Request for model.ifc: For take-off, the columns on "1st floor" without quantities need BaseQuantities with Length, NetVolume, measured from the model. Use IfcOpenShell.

First a look at what the model holds.

```python
import ifcopenshell
import ifcopenshell.util.element
import ifcopenshell.util.unit

model = ifcopenshell.open("model.ifc")
print(model.schema)
for unit_type in ("LENGTHUNIT", "AREAUNIT", "VOLUMEUNIT"):
    print(unit_type, ifcopenshell.util.unit.calculate_unit_scale(model, unit_type))
storey = next(s for s in model.by_type("IfcBuildingStorey") if s.Name == "1st floor")
columns = [e for e in ifcopenshell.util.element.get_decomposition(storey) if e.is_a("IfcColumn")]
for e in sorted(columns, key=lambda e: e.id()):
    print(e.id(), e.is_a(), e.Name, list(ifcopenshell.util.element.get_psets(e, qtos_only=True)), sep=" | ")
```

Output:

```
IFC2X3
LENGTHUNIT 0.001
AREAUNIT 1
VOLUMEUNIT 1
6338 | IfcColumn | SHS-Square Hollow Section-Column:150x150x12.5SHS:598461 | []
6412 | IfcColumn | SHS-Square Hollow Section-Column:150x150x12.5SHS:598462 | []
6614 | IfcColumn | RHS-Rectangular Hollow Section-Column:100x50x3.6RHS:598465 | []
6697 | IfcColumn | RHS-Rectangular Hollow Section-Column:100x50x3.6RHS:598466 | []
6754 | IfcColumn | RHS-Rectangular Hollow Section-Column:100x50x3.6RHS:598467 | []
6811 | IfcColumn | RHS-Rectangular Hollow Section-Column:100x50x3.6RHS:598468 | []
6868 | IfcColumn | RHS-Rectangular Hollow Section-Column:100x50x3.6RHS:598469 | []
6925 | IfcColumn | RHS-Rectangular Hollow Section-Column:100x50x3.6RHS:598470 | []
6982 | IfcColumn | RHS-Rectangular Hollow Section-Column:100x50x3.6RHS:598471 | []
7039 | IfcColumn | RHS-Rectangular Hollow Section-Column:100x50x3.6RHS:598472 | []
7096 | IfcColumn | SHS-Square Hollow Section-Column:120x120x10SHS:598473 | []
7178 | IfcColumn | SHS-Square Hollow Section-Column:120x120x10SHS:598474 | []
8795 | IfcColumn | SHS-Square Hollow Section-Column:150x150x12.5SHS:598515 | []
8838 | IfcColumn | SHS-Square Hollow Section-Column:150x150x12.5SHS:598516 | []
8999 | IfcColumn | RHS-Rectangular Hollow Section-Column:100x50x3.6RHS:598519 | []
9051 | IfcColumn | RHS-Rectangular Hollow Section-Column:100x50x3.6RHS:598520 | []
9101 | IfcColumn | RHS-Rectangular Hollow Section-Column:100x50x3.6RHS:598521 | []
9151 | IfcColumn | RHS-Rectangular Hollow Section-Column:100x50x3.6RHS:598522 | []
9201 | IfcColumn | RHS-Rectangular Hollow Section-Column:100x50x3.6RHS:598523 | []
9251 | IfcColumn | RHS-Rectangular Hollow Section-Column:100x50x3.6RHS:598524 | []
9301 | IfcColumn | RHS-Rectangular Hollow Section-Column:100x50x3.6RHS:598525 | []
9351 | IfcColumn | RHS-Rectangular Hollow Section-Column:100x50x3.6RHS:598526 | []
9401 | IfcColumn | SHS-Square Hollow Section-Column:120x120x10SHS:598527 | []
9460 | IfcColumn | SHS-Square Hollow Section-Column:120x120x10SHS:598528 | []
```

```python
import ifcopenshell
import ifcopenshell.api.pset
import ifcopenshell.geom
import ifcopenshell.util.element
import ifcopenshell.util.shape
import ifcopenshell.util.unit

model = ifcopenshell.open("model.ifc")
unit_scale = ifcopenshell.util.unit.calculate_unit_scale(model)
volume_scale = ifcopenshell.util.unit.calculate_unit_scale(model, "VOLUMEUNIT")
settings = ifcopenshell.geom.settings()

storey = next(s for s in model.by_type("IfcBuildingStorey") if s.Name == "1st floor")
columns = [e for e in ifcopenshell.util.element.get_decomposition(storey) if e.is_a("IfcColumn")]

for e in sorted(columns, key=lambda e: e.id()):
    if ifcopenshell.util.element.get_psets(e, qtos_only=True, should_inherit=False):
        continue
    # Geometry comes back in metres, in the element's own axes.
    shape = ifcopenshell.geom.create_shape(settings, e)
    values = {
        "Length": ifcopenshell.util.shape.get_z(shape.geometry) / unit_scale,
        "NetVolume": ifcopenshell.util.shape.get_volume(shape.geometry) / volume_scale,
    }
    qto = ifcopenshell.api.pset.add_qto(model, product=e, name="BaseQuantities")
    ifcopenshell.api.pset.edit_qto(model, qto=qto, properties=values)
    print(e.id(), {k: round(v, 3) for k, v in values.items()})

model.write("model_v2.ifc")
```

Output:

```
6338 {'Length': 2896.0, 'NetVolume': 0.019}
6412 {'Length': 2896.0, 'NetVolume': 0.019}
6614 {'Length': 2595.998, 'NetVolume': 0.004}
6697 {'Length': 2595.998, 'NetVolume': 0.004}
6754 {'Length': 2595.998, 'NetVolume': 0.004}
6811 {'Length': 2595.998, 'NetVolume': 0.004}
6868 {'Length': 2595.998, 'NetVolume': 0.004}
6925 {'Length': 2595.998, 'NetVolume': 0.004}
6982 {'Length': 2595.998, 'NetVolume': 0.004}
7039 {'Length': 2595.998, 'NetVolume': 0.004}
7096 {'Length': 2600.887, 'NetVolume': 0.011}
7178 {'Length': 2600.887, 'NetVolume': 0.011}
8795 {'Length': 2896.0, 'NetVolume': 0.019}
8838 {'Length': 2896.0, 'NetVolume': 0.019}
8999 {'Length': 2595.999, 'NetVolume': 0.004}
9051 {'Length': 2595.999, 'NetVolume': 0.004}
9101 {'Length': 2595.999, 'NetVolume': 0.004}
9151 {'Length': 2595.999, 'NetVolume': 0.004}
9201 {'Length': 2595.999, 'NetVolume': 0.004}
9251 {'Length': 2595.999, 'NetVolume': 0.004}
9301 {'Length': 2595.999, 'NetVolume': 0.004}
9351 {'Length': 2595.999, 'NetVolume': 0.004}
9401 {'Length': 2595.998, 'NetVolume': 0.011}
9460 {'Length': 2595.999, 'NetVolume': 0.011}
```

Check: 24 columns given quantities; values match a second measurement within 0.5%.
